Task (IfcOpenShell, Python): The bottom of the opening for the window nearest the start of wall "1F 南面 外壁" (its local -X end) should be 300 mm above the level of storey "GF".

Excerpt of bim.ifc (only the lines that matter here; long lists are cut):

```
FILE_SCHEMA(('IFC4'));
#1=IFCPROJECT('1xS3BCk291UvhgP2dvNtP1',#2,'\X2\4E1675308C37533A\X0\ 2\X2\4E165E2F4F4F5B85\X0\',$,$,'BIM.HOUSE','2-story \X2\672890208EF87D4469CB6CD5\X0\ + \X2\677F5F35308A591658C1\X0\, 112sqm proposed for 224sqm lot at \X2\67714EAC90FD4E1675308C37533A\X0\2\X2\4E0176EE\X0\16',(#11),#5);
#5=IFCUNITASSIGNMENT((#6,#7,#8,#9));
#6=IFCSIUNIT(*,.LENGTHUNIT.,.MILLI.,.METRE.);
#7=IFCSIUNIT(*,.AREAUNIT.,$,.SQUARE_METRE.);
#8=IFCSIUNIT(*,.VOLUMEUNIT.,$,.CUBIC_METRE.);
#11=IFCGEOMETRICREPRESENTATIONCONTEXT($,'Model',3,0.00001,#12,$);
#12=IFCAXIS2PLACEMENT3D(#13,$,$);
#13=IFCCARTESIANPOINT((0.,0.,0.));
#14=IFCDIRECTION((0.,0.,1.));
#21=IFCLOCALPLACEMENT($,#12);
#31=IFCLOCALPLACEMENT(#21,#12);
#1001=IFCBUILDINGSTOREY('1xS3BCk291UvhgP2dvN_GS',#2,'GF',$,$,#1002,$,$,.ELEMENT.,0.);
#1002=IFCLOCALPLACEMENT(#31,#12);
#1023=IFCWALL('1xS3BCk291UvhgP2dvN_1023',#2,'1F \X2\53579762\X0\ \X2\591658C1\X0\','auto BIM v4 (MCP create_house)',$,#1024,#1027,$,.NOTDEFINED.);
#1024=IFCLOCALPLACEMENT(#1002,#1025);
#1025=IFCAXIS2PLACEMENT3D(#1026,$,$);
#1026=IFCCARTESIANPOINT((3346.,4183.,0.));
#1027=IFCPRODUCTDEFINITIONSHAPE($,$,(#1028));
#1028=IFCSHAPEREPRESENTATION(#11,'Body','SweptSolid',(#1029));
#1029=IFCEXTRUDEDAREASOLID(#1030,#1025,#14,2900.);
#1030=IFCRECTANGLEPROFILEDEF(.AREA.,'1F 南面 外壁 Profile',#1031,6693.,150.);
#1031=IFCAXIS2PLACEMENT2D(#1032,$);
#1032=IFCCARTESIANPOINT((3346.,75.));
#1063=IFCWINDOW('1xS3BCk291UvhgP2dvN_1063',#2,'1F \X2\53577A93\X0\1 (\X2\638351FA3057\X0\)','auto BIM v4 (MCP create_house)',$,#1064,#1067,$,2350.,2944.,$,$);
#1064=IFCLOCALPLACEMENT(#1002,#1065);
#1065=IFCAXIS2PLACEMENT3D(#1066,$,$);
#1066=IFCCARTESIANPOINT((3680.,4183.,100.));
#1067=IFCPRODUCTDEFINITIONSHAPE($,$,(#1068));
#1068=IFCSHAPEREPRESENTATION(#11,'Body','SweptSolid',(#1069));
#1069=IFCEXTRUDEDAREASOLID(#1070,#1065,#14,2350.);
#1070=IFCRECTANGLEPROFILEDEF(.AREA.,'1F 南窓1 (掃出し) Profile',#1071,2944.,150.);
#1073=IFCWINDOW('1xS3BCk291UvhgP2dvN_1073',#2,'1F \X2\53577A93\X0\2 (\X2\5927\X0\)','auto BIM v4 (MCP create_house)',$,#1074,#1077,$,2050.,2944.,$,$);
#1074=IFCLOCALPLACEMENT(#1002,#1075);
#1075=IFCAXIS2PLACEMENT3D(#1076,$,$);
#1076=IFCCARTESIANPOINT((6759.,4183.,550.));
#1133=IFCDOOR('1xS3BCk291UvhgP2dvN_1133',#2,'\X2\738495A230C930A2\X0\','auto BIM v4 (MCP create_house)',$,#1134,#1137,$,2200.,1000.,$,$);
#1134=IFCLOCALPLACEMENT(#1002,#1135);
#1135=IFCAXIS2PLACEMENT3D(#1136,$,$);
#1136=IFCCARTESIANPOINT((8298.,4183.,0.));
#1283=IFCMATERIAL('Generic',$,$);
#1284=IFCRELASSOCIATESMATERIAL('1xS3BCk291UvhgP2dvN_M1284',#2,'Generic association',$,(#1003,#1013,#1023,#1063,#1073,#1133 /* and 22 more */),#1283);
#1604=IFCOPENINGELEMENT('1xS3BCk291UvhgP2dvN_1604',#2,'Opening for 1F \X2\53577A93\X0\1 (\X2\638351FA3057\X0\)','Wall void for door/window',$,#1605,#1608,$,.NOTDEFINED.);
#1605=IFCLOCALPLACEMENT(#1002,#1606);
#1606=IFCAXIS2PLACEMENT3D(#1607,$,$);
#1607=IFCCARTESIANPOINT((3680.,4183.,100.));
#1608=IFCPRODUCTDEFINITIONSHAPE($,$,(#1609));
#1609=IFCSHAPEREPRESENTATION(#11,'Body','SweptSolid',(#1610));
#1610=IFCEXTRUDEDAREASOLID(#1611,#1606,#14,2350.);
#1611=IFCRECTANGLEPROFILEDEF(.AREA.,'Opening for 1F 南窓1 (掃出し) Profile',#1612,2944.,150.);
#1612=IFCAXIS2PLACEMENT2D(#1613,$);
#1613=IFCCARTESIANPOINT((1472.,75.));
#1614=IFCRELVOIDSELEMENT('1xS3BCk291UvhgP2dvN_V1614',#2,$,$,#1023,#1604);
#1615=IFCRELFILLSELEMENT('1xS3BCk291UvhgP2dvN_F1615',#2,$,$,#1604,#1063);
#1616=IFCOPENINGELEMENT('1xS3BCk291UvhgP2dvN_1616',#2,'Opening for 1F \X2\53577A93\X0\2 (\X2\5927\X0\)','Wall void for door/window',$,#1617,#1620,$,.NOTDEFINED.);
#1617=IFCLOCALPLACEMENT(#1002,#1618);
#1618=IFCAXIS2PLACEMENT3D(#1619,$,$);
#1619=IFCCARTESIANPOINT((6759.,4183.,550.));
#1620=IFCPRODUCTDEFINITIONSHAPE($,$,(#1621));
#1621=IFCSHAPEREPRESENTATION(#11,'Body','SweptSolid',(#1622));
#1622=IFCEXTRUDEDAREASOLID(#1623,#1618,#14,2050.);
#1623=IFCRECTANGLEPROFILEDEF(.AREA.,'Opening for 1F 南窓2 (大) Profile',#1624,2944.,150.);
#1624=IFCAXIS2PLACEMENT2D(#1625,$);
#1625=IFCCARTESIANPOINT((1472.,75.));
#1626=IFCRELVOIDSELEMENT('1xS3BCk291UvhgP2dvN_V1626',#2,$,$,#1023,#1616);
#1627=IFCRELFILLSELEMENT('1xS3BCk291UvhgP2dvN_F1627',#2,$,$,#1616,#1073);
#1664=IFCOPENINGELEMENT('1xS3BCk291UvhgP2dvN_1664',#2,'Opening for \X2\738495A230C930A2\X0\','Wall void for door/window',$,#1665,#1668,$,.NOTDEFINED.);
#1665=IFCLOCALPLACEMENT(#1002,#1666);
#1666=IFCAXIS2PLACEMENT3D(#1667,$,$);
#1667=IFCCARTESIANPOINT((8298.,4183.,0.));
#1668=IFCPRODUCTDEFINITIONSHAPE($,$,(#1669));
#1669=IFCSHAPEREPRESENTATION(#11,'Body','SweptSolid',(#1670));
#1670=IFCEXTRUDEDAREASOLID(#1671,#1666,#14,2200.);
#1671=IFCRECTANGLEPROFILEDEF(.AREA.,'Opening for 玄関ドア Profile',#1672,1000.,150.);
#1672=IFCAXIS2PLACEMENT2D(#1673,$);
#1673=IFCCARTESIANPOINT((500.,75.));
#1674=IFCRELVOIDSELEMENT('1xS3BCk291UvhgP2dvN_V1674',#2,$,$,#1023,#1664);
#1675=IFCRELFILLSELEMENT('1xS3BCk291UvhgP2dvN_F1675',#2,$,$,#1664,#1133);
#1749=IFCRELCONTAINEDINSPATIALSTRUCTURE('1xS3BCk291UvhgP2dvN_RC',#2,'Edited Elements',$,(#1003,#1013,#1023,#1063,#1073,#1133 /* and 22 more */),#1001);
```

```python
import numpy as np
import ifcopenshell
import ifcopenshell.api.geometry
import ifcopenshell.geom
import ifcopenshell.util.element
import ifcopenshell.util.placement
import ifcopenshell.util.shape
import ifcopenshell.util.unit

model = ifcopenshell.open("bim.ifc")
unit_scale = ifcopenshell.util.unit.calculate_unit_scale(model)

window = model.by_guid("1xS3BCk291UvhgP2dvN_1063")
opening = window.FillsVoids[0].RelatingOpeningElement
storey = ifcopenshell.util.element.get_container(window, ifc_class="IfcBuildingStorey")
level = ifcopenshell.util.placement.get_local_placement(storey.ObjectPlacement)[2, 3]

# The opening's origin need not be at the sill, so measure its lowest point.
shape = ifcopenshell.geom.create_shape(ifcopenshell.geom.settings(), opening)
bottom = ifcopenshell.util.shape.get_shape_bottom_elevation(shape, shape.geometry) / unit_scale
dz = level + 0.3 / unit_scale - bottom

shift = np.array([0.0, 0.0, dz])
# The window is not placed relative to its opening, so move both.
for product in (opening, window):
    matrix = ifcopenshell.util.placement.get_local_placement(product.ObjectPlacement)
    matrix[:3, 3] += shift
    ifcopenshell.api.geometry.edit_object_placement(model, product=product, matrix=matrix, is_si=False)

print(f"moved by {dz * unit_scale:+.3f} m")

model.write("bim_updated.ifc")
```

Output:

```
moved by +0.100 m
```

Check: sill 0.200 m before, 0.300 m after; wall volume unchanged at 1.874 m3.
